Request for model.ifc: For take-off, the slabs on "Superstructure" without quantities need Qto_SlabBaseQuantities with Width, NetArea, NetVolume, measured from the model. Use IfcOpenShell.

First a look at what the model holds.

```python
import ifcopenshell
import ifcopenshell.util.element
import ifcopenshell.util.unit

model = ifcopenshell.open("model.ifc")
print(model.schema)
for unit_type in ("LENGTHUNIT", "AREAUNIT", "VOLUMEUNIT"):
    print(unit_type, ifcopenshell.util.unit.calculate_unit_scale(model, unit_type))
storey = next(s for s in model.by_type("IfcBuildingStorey") if s.Name == "Superstructure")
slabs = [e for e in ifcopenshell.util.element.get_decomposition(storey) if e.is_a("IfcSlab")]
for e in sorted(slabs, key=lambda e: e.id()):
    print(e.id(), e.is_a(), e.Name, list(ifcopenshell.util.element.get_psets(e, qtos_only=True)), sep=" | ")
```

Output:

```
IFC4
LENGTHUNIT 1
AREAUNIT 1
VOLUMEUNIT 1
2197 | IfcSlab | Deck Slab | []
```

```python
import ifcopenshell
import ifcopenshell.api.pset
import ifcopenshell.geom
import ifcopenshell.util.element
import ifcopenshell.util.shape
import ifcopenshell.util.unit

model = ifcopenshell.open("model.ifc")
unit_scale = ifcopenshell.util.unit.calculate_unit_scale(model)
area_scale = ifcopenshell.util.unit.calculate_unit_scale(model, "AREAUNIT")
volume_scale = ifcopenshell.util.unit.calculate_unit_scale(model, "VOLUMEUNIT")
settings = ifcopenshell.geom.settings()

storey = next(s for s in model.by_type("IfcBuildingStorey") if s.Name == "Superstructure")
slabs = [e for e in ifcopenshell.util.element.get_decomposition(storey) if e.is_a("IfcSlab")]

for e in sorted(slabs, key=lambda e: e.id()):
    if ifcopenshell.util.element.get_psets(e, qtos_only=True, should_inherit=False):
        continue
    # Geometry comes back in metres, in the element's own axes.
    shape = ifcopenshell.geom.create_shape(settings, e)
    values = {
        "Width": ifcopenshell.util.shape.get_z(shape.geometry) / unit_scale,
        "NetArea": ifcopenshell.util.shape.get_footprint_area(shape.geometry) / area_scale,
        "NetVolume": ifcopenshell.util.shape.get_volume(shape.geometry) / volume_scale,
    }
    qto = ifcopenshell.api.pset.add_qto(model, product=e, name="Qto_SlabBaseQuantities")
    ifcopenshell.api.pset.edit_qto(model, qto=qto, properties=values)
    print(e.id(), {k: round(v, 3) for k, v in values.items()})

model.write("model-out.ifc")
```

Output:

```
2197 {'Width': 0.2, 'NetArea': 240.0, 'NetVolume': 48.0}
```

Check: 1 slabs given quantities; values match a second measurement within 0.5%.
